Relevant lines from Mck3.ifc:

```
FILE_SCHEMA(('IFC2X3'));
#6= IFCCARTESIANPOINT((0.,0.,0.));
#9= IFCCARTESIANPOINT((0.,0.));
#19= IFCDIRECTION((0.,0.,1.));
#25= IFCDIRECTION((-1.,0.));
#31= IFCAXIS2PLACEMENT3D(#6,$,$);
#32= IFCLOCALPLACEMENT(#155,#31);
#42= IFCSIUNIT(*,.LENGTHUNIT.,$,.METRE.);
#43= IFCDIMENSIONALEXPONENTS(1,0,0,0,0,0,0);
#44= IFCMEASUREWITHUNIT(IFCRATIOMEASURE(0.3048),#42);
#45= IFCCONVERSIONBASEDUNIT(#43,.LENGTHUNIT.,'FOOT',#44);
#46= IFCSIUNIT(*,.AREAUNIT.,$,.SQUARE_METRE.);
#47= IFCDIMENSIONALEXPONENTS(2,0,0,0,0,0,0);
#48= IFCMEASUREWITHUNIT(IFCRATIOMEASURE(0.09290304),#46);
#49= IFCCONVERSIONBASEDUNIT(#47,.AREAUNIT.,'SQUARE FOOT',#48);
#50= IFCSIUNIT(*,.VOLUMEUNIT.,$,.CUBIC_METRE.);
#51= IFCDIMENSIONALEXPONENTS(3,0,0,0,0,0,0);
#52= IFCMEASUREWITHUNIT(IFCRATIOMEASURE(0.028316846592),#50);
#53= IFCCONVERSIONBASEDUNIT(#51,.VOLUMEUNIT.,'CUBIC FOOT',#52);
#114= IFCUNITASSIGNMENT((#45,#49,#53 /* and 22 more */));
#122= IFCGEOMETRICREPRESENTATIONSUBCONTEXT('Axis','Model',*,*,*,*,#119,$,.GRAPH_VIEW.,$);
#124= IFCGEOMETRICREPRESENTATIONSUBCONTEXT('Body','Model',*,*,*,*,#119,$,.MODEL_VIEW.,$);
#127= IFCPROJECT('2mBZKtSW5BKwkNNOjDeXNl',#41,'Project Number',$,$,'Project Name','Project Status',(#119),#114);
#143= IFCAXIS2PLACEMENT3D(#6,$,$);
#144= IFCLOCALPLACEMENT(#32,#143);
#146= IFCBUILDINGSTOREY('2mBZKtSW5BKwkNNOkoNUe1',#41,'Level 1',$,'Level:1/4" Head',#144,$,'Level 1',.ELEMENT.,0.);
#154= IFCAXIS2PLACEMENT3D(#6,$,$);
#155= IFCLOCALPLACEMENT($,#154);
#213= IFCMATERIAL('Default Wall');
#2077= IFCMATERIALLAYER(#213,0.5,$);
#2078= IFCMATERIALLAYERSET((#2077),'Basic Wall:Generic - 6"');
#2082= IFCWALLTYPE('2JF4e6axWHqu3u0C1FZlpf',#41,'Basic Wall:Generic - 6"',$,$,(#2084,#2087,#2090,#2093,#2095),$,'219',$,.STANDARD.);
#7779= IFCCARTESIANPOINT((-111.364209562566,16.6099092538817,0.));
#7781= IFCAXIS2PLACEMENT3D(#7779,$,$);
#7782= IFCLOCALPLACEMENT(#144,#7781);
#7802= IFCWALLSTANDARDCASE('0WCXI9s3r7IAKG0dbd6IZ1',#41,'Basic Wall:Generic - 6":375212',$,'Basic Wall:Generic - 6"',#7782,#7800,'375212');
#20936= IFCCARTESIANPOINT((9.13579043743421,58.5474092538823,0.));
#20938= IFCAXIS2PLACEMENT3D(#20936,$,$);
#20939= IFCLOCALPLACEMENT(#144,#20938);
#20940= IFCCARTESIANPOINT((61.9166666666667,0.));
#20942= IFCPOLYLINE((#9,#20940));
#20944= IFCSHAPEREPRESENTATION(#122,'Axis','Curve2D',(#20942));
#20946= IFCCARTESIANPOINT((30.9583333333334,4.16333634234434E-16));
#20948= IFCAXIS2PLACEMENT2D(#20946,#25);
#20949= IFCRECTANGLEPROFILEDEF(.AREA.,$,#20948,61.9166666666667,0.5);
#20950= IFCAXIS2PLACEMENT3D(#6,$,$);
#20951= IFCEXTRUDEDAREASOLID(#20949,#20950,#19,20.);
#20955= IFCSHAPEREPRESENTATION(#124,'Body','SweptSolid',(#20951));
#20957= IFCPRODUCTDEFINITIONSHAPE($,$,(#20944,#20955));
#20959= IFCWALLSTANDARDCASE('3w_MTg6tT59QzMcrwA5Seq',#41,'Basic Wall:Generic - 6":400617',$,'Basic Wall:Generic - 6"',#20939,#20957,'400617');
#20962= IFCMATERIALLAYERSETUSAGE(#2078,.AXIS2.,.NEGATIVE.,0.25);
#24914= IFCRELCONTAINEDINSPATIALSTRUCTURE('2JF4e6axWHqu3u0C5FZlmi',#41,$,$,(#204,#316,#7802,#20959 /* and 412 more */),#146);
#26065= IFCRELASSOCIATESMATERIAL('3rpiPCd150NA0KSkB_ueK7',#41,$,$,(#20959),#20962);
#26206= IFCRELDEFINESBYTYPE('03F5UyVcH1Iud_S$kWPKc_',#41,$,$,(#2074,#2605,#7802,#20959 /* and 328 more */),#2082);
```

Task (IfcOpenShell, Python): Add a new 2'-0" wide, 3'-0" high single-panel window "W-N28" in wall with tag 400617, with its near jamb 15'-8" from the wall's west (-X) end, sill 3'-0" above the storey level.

```python
import numpy as np
import ifcopenshell
import ifcopenshell.api.feature
import ifcopenshell.api.geometry
import ifcopenshell.api.root
import ifcopenshell.api.spatial
import ifcopenshell.api.type
import ifcopenshell.geom
import ifcopenshell.util.element
import ifcopenshell.util.placement
import ifcopenshell.util.representation
import ifcopenshell.util.shape
import ifcopenshell.util.unit

model = ifcopenshell.open("Mck3.ifc")
unit_scale = ifcopenshell.util.unit.calculate_unit_scale(model)
settings = ifcopenshell.geom.settings()


def volume(element):
    """Net volume in cubic metres, openings subtracted."""
    shape = ifcopenshell.geom.create_shape(settings, element)
    return ifcopenshell.util.shape.get_volume(shape.geometry)


wall = model.by_id(20959)
storey = ifcopenshell.util.element.get_container(wall, ifc_class="IfcBuildingStorey")
context = ifcopenshell.util.representation.get_context(model, "Model", "Body", "MODEL_VIEW")
before = volume(wall)

width, height, from_end, sill = 0.6096, 0.9144, 4.7752, 0.9144  # metres

# The wall runs along its own X axis, and the end named is its -X end.
wall_shape = ifcopenshell.geom.create_shape(settings, wall)
x, y, z = ifcopenshell.util.shape.get_vertices(wall_shape.geometry).T
start = x.min() + from_end
face, thickness = float(y.min()), float(y.max() - y.min())
wall_matrix = ifcopenshell.util.placement.get_local_placement(wall.ObjectPlacement)
level = ifcopenshell.util.placement.get_local_placement(storey.ObjectPlacement)[2, 3]


def in_wall(x, y):
    """Placement at x, y metres in the wall's axes, at sill height."""
    matrix = wall_matrix.copy()
    matrix[:, 3] = wall_matrix @ np.array([x / unit_scale, y / unit_scale, 0.0, 1.0])
    matrix[2, 3] = level + sill / unit_scale
    return matrix


# Opening: a box that overshoots both wall faces by 50 mm.
opening = ifcopenshell.api.root.create_entity(model, ifc_class="IfcOpeningElement")
box = ifcopenshell.api.geometry.add_wall_representation(
    model, context=context, length=width, height=height, thickness=thickness + 0.1
)
ifcopenshell.api.geometry.assign_representation(model, product=opening, representation=box)
ifcopenshell.api.geometry.edit_object_placement(model, product=opening, matrix=in_wall(start, face - 0.05), is_si=False)
ifcopenshell.api.feature.add_feature(model, feature=opening, element=wall)

window = ifcopenshell.api.root.create_entity(model, ifc_class="IfcWindow", name="W-N28")
window.OverallWidth, window.OverallHeight = width / unit_scale, height / unit_scale
body = ifcopenshell.api.geometry.add_window_representation(
    model,
    context=context,
    overall_width=window.OverallWidth,
    overall_height=window.OverallHeight,
    partition_type="SINGLE_PANEL",
)
ifcopenshell.api.geometry.assign_representation(model, product=window, representation=body)
ifcopenshell.api.spatial.assign_container(model, products=[window], relating_structure=storey)
fills = ifcopenshell.api.feature.add_filling(model, opening=opening, element=window)
fills.OwnerHistory = window.OwnerHistory  # required in IFC2X3

# IFC2X3 keeps the operation on the window style.
style = ifcopenshell.api.root.create_entity(model, ifc_class="IfcWindowStyle", name="W-N28")
style.OperationType, style.ConstructionType = "SINGLE_PANEL", "NOTDEFINED"
style.ParameterTakesPrecedence = style.Sizeable = False
ifcopenshell.api.type.assign_type(model, related_objects=[window], relating_type=style)

# Centre the window in the wall's thickness.
ifcopenshell.api.geometry.edit_object_placement(model, product=window, matrix=in_wall(start, face), is_si=False)
window_shape = ifcopenshell.geom.create_shape(settings, window)
depth = ifcopenshell.util.shape.get_vertices(window_shape.geometry)[:, 1]
offset = face + thickness / 2 - (depth.min() + depth.max()) / 2
ifcopenshell.api.geometry.edit_object_placement(model, product=window, matrix=in_wall(start, offset), is_si=False)

after = volume(wall)

print(f"wall volume {before:.3f} -> {after:.3f} m3")

model.write("Mck3_updated.ifc")
```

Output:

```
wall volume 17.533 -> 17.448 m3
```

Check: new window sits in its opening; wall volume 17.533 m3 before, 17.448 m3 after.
